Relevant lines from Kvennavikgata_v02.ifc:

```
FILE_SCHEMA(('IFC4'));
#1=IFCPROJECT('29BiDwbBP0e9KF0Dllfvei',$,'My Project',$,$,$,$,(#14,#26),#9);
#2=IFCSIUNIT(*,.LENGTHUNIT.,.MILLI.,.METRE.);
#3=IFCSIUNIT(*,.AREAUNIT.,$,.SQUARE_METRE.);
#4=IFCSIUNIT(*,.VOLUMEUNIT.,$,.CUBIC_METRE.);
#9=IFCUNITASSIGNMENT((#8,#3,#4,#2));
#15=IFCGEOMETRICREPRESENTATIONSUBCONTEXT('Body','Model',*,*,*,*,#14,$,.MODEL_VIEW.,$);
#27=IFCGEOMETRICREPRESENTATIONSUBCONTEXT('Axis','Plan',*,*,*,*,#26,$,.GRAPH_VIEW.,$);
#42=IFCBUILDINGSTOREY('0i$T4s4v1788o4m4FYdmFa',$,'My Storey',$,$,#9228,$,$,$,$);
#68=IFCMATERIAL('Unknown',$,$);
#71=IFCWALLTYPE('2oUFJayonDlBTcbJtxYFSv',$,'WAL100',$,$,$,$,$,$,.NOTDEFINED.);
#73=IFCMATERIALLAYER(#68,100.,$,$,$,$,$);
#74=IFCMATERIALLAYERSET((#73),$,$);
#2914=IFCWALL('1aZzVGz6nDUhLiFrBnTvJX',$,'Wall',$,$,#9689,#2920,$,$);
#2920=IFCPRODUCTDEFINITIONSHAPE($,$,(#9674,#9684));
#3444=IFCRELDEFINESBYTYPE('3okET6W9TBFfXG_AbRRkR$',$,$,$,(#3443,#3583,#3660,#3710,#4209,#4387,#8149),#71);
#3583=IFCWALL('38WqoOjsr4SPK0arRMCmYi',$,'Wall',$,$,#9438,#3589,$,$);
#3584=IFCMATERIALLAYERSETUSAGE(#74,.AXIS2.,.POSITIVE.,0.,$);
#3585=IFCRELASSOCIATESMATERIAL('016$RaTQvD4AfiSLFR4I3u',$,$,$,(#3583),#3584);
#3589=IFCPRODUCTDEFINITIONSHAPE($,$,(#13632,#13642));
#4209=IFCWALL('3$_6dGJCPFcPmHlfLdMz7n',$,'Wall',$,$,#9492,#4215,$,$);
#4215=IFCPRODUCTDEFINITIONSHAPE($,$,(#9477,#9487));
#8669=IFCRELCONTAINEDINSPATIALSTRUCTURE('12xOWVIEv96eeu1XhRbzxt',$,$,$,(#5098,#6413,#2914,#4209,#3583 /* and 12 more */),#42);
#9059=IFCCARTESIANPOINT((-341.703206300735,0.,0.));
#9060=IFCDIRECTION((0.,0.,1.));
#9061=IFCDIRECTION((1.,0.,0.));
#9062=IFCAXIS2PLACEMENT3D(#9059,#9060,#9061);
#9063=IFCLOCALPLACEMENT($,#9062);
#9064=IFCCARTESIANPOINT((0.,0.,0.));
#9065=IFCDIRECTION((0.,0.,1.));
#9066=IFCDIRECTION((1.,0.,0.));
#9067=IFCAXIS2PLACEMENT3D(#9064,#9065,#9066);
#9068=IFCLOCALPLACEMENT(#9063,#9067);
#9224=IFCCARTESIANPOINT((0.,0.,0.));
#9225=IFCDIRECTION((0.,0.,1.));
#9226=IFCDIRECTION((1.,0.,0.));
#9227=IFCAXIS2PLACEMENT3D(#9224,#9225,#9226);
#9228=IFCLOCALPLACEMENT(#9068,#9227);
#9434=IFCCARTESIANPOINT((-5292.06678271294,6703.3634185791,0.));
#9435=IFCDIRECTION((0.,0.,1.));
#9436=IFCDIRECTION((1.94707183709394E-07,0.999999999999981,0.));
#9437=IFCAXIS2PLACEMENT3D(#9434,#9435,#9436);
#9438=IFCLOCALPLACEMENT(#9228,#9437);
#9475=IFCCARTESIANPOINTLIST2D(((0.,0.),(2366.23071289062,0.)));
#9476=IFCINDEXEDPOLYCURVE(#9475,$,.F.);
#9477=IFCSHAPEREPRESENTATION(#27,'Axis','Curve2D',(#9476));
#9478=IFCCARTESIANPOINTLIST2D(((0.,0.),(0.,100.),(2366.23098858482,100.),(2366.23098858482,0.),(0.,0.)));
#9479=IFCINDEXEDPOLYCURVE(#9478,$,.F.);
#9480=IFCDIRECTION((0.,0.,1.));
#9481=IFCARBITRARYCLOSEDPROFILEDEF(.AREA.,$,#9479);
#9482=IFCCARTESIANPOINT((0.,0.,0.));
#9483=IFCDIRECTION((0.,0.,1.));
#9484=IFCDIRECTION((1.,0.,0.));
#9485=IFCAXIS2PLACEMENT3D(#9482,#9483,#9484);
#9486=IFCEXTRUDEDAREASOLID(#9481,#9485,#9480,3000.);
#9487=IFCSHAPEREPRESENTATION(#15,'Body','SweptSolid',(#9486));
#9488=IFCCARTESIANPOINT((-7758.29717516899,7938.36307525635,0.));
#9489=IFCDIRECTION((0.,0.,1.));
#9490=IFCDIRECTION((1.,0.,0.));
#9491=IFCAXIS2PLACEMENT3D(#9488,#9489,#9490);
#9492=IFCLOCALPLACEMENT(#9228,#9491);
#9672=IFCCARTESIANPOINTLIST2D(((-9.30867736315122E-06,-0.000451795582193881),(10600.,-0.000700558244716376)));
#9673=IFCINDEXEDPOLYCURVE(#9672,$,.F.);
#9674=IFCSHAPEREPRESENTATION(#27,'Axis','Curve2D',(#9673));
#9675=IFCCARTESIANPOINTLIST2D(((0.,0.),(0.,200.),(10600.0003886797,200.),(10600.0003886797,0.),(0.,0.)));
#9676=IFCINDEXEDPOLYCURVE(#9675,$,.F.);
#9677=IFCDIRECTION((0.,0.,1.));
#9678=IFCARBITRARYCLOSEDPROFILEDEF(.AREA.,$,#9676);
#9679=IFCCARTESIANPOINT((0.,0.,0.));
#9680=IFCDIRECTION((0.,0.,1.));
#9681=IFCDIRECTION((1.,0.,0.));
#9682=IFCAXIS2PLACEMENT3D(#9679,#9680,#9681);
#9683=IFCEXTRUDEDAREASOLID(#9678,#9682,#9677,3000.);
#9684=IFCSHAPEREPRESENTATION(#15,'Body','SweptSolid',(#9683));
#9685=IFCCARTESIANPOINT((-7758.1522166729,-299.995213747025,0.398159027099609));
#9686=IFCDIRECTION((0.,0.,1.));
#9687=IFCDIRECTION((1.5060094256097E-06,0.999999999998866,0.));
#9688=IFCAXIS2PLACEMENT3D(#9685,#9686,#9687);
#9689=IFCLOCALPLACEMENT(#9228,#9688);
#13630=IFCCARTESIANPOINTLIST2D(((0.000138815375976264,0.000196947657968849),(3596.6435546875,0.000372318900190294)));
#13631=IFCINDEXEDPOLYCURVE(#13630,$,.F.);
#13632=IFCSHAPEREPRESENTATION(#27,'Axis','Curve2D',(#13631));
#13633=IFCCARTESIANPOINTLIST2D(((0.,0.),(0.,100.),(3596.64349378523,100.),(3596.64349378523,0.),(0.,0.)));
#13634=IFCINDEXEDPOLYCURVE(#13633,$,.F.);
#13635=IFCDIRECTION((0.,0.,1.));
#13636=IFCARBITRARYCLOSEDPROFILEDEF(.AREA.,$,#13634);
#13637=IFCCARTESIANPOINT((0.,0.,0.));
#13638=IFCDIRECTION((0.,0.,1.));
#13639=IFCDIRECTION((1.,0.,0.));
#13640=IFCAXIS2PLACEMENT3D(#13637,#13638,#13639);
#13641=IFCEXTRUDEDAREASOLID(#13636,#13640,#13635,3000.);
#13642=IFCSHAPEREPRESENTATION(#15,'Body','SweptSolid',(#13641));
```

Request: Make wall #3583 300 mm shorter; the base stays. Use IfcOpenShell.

```python
import ifcopenshell
import ifcopenshell.geom
import ifcopenshell.util.representation
import ifcopenshell.util.shape

model = ifcopenshell.open("Kvennavikgata_v02.ifc")
settings = ifcopenshell.geom.settings()


def volume(element):
    """Net volume in cubic metres, openings subtracted."""
    shape = ifcopenshell.geom.create_shape(settings, element)
    return ifcopenshell.util.shape.get_volume(shape.geometry)


wall = model.by_id(3583)
before = volume(wall)

body = ifcopenshell.util.representation.get_representation(wall, "Model", "Body")
solid = body.Items[0]
old_height = solid.Depth
solid.Depth -= 300.0
after = volume(wall)

print(f"height {old_height:g} -> {solid.Depth:g}, volume {before:.3f} -> {after:.3f} m3")

model.write("Kvennavikgata_v02_updated.ifc")
```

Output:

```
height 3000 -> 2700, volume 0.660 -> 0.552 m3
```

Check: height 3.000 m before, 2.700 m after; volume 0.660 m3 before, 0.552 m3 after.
